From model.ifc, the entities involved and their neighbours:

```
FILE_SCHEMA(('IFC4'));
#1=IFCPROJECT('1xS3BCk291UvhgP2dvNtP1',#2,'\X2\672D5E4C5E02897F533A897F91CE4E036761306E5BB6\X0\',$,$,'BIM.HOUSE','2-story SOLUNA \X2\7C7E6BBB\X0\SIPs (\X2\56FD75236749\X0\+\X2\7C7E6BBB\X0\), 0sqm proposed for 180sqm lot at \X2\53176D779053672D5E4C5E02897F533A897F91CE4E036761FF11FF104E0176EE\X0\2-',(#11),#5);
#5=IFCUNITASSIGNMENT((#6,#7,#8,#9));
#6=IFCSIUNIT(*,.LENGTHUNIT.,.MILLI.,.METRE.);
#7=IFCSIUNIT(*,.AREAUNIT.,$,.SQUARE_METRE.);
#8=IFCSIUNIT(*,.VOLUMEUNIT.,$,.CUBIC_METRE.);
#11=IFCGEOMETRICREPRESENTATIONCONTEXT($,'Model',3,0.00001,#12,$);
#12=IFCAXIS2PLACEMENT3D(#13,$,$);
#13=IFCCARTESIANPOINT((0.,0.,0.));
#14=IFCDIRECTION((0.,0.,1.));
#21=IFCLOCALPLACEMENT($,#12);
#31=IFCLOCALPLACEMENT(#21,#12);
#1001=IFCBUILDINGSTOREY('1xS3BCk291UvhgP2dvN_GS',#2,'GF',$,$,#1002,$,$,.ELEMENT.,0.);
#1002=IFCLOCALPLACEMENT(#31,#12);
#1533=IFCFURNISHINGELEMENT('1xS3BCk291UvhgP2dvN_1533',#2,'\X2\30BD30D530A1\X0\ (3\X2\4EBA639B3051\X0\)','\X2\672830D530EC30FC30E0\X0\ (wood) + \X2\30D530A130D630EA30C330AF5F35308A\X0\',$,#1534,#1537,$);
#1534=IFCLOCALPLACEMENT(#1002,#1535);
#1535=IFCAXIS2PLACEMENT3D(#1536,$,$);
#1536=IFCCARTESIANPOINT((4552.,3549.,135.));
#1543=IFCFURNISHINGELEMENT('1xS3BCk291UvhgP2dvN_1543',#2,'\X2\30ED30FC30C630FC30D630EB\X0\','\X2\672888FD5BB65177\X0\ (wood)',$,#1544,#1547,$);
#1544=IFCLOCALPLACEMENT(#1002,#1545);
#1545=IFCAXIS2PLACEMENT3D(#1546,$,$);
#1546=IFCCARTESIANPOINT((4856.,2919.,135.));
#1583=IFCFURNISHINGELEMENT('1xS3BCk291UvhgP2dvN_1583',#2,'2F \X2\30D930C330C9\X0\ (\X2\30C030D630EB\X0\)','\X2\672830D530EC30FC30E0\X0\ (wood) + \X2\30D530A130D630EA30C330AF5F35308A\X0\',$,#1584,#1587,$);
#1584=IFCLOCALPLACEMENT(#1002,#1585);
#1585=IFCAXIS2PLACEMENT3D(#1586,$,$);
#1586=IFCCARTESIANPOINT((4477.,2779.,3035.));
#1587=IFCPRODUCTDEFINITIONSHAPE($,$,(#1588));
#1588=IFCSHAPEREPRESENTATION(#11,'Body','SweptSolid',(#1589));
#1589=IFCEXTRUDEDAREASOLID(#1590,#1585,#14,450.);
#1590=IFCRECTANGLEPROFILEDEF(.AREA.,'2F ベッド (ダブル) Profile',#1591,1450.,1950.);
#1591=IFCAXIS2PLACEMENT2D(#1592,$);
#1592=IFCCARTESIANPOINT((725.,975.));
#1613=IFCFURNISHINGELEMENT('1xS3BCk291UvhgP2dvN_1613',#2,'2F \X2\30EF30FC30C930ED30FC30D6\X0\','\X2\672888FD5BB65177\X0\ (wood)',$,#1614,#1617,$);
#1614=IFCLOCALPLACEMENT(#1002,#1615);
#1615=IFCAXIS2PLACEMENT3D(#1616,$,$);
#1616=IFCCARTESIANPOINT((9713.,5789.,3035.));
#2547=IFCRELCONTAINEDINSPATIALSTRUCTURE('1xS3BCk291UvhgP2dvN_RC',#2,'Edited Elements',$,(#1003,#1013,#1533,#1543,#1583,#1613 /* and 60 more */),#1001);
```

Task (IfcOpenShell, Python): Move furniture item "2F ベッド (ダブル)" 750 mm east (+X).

```python
import ifcopenshell
import ifcopenshell.api.geometry
import ifcopenshell.util.placement

model = ifcopenshell.open("model.ifc")

item = model.by_guid("1xS3BCk291UvhgP2dvN_1583")
matrix = ifcopenshell.util.placement.get_local_placement(item.ObjectPlacement)
matrix[0, 3] += 750.0
ifcopenshell.api.geometry.edit_object_placement(model, product=item, matrix=matrix, is_si=False)

print(ifcopenshell.util.placement.get_local_placement(item.ObjectPlacement).round(3) + 0.0)

model.write("model_updated.ifc")
```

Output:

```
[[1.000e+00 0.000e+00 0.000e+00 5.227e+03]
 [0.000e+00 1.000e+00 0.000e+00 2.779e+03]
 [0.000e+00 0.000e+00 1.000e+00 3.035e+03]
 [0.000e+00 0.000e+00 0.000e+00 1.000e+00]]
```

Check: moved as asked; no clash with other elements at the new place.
